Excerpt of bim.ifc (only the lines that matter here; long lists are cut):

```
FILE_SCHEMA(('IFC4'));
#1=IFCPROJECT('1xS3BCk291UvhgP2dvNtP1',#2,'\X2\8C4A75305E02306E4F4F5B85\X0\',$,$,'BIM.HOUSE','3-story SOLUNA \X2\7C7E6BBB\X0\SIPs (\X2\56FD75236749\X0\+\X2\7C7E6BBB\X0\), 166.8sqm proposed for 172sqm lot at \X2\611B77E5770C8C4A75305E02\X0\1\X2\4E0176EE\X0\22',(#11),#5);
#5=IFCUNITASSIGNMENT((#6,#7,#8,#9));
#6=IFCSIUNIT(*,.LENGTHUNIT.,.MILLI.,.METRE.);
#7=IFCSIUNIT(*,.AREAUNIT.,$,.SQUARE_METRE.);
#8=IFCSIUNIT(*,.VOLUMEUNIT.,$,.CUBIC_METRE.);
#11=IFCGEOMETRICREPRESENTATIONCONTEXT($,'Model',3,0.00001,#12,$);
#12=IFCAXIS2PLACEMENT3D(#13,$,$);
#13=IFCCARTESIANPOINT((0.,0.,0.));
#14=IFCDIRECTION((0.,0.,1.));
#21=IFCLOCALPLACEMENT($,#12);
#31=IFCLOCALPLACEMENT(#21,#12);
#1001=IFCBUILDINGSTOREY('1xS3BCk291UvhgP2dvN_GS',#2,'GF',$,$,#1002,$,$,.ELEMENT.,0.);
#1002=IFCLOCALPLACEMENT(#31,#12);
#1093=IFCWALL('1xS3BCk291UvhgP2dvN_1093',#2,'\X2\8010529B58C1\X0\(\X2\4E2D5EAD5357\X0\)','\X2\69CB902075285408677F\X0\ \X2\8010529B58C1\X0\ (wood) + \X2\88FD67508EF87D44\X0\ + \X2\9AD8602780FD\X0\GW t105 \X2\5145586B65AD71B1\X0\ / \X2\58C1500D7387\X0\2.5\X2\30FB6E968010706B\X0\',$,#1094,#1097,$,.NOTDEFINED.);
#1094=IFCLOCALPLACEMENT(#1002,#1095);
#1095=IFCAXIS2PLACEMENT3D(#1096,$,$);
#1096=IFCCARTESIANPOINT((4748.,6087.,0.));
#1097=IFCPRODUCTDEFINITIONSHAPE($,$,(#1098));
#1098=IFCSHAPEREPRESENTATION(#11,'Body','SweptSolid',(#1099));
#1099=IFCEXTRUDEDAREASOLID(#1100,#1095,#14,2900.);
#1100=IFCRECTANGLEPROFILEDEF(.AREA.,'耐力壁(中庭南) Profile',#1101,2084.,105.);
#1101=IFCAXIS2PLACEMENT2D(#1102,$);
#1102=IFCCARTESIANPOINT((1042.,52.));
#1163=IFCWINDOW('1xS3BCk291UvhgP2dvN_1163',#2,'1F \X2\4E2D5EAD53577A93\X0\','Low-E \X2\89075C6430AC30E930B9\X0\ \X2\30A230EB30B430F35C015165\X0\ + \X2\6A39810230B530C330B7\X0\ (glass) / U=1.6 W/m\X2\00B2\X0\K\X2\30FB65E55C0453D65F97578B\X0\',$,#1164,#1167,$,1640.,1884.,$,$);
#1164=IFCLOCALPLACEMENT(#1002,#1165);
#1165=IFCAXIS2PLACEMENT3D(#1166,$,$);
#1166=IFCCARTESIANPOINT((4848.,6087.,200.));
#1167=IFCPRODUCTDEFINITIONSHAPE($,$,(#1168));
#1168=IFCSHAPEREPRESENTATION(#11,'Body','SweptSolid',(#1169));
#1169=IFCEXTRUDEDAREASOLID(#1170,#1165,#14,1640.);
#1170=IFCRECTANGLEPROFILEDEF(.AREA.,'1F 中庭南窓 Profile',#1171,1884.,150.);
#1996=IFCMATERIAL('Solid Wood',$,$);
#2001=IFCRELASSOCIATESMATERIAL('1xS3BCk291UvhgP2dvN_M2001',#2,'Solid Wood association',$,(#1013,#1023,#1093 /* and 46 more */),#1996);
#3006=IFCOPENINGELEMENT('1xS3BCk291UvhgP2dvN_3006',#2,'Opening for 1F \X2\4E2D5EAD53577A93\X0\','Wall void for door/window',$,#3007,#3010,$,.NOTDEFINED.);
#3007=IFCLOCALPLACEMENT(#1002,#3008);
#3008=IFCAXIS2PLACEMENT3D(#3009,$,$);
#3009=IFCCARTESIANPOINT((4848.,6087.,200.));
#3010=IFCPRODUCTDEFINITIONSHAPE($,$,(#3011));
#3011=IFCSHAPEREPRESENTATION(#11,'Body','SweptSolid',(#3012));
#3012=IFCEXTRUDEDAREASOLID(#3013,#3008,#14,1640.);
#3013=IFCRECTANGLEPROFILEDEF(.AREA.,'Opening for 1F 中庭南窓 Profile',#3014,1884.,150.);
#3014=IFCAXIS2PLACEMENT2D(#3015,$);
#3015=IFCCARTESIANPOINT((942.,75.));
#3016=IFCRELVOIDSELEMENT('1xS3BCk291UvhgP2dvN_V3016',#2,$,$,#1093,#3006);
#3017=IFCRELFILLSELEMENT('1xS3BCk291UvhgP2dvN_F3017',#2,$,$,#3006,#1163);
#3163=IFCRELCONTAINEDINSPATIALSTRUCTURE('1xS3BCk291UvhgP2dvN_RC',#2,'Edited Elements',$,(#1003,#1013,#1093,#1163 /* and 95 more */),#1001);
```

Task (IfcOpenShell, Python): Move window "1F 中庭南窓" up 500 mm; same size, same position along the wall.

```python
import numpy as np
import ifcopenshell
import ifcopenshell.api.geometry
import ifcopenshell.util.placement
import ifcopenshell.util.unit

model = ifcopenshell.open("bim.ifc")
unit_scale = ifcopenshell.util.unit.calculate_unit_scale(model)

window = model.by_id(1163)
opening = window.FillsVoids[0].RelatingOpeningElement
dz = 500.0

shift = np.array([0.0, 0.0, dz])
# The window is not placed relative to its opening, so move both.
for product in (opening, window):
    matrix = ifcopenshell.util.placement.get_local_placement(product.ObjectPlacement)
    matrix[:3, 3] += shift
    ifcopenshell.api.geometry.edit_object_placement(model, product=product, matrix=matrix, is_si=False)

print(f"moved by {dz * unit_scale:+.3f} m")

model.write("bim_v2.ifc")
```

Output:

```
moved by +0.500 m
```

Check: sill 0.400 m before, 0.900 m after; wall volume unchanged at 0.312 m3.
